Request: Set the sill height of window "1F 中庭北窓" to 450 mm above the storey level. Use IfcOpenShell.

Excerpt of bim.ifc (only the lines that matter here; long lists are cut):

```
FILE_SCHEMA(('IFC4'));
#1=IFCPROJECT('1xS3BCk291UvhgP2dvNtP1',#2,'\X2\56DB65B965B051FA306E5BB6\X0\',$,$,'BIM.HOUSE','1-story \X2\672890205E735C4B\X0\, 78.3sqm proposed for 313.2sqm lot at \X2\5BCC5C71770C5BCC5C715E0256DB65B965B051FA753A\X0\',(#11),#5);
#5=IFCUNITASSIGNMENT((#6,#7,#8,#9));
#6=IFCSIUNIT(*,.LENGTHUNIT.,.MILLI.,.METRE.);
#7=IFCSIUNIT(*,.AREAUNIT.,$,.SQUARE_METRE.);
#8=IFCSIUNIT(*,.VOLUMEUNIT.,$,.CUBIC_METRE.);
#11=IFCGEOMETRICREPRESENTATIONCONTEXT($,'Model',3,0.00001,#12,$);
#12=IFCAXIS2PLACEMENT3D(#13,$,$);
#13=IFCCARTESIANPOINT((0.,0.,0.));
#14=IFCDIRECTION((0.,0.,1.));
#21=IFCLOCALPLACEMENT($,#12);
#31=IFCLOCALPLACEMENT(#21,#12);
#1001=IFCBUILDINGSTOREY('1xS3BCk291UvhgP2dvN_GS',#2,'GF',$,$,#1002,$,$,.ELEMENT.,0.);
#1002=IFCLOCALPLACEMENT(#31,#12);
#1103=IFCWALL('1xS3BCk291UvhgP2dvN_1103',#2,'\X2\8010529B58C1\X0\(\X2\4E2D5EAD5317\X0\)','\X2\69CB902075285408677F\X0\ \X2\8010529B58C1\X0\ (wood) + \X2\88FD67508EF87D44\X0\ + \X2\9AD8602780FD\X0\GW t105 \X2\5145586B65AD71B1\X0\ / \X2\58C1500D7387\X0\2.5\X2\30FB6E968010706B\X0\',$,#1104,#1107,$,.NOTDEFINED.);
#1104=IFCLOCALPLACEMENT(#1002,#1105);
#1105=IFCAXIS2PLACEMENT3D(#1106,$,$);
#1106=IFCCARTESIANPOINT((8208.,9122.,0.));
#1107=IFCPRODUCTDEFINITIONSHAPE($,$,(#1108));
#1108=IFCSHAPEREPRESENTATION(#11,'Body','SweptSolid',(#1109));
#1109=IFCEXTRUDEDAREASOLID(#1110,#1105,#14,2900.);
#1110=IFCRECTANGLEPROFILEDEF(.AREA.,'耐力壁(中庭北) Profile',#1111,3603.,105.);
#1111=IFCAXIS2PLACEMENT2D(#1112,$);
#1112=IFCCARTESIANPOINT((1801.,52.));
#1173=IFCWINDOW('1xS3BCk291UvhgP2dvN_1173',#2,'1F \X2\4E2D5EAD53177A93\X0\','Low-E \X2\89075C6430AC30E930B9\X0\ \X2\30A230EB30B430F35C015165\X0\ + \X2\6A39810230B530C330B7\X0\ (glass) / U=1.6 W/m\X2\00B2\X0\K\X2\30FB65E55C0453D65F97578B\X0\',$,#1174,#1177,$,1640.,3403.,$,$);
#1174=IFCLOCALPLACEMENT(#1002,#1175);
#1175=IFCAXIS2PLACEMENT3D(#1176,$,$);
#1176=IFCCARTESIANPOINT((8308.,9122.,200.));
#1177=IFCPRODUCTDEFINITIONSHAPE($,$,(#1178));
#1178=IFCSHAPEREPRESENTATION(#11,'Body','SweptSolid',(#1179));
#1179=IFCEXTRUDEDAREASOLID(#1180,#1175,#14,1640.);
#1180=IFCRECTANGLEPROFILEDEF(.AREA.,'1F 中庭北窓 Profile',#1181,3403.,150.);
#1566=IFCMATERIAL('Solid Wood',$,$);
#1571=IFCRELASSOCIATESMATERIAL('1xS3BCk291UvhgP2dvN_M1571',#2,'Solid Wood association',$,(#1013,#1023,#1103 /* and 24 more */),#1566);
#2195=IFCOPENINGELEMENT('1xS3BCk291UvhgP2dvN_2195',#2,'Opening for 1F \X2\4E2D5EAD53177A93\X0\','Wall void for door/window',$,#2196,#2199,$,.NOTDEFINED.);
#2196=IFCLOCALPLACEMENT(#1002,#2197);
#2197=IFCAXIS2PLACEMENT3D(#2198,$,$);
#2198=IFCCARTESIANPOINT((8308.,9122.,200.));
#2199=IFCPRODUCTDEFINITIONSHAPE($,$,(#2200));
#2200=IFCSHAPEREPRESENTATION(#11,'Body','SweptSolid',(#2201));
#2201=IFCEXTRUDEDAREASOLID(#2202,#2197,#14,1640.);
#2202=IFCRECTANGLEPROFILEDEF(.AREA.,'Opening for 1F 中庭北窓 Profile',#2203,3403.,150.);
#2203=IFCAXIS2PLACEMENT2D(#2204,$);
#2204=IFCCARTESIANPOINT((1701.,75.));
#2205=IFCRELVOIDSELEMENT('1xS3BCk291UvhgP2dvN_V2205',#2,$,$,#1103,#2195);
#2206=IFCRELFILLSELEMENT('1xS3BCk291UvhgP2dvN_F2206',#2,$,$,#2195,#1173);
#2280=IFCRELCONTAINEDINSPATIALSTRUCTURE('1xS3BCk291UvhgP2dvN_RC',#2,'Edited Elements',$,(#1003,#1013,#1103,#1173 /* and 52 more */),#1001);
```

```python
import numpy as np
import ifcopenshell
import ifcopenshell.api.geometry
import ifcopenshell.geom
import ifcopenshell.util.element
import ifcopenshell.util.placement
import ifcopenshell.util.shape
import ifcopenshell.util.unit

model = ifcopenshell.open("bim.ifc")
unit_scale = ifcopenshell.util.unit.calculate_unit_scale(model)

window = model.by_id(1173)
opening = window.FillsVoids[0].RelatingOpeningElement
storey = ifcopenshell.util.element.get_container(window, ifc_class="IfcBuildingStorey")
level = ifcopenshell.util.placement.get_local_placement(storey.ObjectPlacement)[2, 3]

# The opening's origin need not be at the sill, so measure its lowest point.
shape = ifcopenshell.geom.create_shape(ifcopenshell.geom.settings(), opening)
bottom = ifcopenshell.util.shape.get_shape_bottom_elevation(shape, shape.geometry) / unit_scale
dz = level + 450.0 - bottom

shift = np.array([0.0, 0.0, dz])
# The window is not placed relative to its opening, so move both.
for product in (opening, window):
    matrix = ifcopenshell.util.placement.get_local_placement(product.ObjectPlacement)
    matrix[:3, 3] += shift
    ifcopenshell.api.geometry.edit_object_placement(model, product=product, matrix=matrix, is_si=False)

print(f"moved by {dz * unit_scale:+.3f} m")

model.write("bim_v2.ifc")
```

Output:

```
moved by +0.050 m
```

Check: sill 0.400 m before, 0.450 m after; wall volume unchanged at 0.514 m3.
